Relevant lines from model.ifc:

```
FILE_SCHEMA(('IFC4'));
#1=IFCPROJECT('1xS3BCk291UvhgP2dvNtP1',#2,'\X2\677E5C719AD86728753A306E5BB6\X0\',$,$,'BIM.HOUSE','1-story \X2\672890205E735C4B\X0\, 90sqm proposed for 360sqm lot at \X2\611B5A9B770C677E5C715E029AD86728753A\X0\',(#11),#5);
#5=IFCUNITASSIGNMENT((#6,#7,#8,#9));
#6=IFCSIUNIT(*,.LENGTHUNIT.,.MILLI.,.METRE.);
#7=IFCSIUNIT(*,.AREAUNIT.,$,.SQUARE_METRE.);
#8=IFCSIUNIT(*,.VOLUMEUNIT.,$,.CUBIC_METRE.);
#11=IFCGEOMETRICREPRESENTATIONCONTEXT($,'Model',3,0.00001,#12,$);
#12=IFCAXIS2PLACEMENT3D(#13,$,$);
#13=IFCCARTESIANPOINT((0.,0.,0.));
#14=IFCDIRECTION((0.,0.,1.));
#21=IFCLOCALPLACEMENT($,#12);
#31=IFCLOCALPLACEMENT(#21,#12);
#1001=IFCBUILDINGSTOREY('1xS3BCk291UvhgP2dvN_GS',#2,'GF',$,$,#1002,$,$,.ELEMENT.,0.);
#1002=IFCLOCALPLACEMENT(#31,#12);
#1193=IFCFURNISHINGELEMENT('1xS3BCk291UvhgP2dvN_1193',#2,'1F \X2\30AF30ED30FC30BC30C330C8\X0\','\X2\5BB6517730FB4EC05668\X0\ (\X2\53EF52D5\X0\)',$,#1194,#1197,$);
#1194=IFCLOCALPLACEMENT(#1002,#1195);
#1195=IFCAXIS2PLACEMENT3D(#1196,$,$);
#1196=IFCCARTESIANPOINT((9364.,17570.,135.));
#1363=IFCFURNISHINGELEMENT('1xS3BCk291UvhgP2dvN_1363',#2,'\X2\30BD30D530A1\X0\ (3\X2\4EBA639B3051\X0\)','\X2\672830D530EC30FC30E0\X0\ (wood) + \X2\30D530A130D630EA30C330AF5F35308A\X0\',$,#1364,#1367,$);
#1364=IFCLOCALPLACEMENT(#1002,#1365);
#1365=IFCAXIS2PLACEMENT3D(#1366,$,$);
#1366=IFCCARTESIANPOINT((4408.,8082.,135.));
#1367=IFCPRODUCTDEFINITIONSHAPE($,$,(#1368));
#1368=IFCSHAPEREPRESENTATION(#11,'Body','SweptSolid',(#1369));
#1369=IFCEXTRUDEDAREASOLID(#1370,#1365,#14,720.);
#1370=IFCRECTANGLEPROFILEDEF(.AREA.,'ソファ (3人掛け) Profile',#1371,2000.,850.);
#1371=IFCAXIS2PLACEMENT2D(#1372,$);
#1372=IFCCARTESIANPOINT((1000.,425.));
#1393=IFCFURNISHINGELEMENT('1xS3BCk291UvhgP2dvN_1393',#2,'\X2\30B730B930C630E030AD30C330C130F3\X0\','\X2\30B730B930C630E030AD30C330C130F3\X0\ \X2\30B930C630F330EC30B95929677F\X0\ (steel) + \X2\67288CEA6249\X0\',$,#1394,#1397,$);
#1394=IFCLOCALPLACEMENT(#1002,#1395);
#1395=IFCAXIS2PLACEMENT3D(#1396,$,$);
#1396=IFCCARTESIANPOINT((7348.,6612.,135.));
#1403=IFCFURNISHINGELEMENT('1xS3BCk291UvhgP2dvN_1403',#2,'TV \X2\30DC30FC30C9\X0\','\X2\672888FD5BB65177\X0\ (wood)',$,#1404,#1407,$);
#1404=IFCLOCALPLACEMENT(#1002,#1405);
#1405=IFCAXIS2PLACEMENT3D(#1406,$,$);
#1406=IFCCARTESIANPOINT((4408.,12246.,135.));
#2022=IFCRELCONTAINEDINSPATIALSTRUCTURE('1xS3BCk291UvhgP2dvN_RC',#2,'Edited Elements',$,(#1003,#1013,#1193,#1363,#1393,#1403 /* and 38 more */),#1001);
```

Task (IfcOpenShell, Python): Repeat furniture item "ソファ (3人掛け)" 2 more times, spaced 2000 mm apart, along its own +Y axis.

```python
import ifcopenshell
import ifcopenshell.api.geometry
import ifcopenshell.api.root
import ifcopenshell.util.element
import ifcopenshell.util.placement
import ifcopenshell.util.unit

model = ifcopenshell.open("model.ifc")
unit_scale = ifcopenshell.util.unit.calculate_unit_scale(model)


def reuse_history(source, copy):
    """copy_class also copies each property set's owner history, people and application; keep the originals."""
    for rel in copy.IsDefinedBy:
        if rel.is_a("IfcRelDefinesByProperties") and (history := rel.RelatingPropertyDefinition.OwnerHistory):
            rel.RelatingPropertyDefinition.OwnerHistory = source.OwnerHistory
            ifcopenshell.util.element.remove_deep2(model, history)


source = model.by_guid("1xS3BCk291UvhgP2dvN_1363")
base = ifcopenshell.util.placement.get_local_placement(source.ObjectPlacement)
step = base[:3, 1] * 2 / unit_scale

for i in range(1, 3):
    copy = ifcopenshell.api.root.copy_class(model, product=source)
    copy.Representation = ifcopenshell.util.element.copy_deep(
        model, source.Representation, exclude=["IfcGeometricRepresentationContext", "IfcRepresentationMap"]
    )
    reuse_history(source, copy)
    matrix = base.copy()
    matrix[:3, 3] += i * step
    print("added at", matrix[:3, 3].round(3) + 0.0)
    ifcopenshell.api.geometry.edit_object_placement(model, product=copy, matrix=matrix, is_si=False)

model.write("model_edited.ifc")
```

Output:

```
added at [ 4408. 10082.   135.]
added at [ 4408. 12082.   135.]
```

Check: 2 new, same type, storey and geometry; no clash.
